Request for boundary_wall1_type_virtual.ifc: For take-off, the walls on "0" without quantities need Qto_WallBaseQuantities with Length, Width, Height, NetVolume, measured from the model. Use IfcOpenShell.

First a look at what the model holds.

```python
import ifcopenshell
import ifcopenshell.util.element
import ifcopenshell.util.unit

model = ifcopenshell.open("boundary_wall1_type_virtual.ifc")
print(model.schema)
for unit_type in ("LENGTHUNIT", "AREAUNIT", "VOLUMEUNIT"):
    print(unit_type, ifcopenshell.util.unit.calculate_unit_scale(model, unit_type))
storey = next(s for s in model.by_type("IfcBuildingStorey") if s.Name == "0")
walls = [e for e in ifcopenshell.util.element.get_decomposition(storey) if e.is_a("IfcWall")]
for e in sorted(walls, key=lambda e: e.id()):
    print(e.id(), e.is_a(), e.Name, list(ifcopenshell.util.element.get_psets(e, qtos_only=True)), sep=" | ")
```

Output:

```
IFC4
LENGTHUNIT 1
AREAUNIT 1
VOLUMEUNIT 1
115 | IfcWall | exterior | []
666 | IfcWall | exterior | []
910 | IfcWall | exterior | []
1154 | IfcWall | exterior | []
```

```python
import ifcopenshell
import ifcopenshell.api.pset
import ifcopenshell.geom
import ifcopenshell.util.element
import ifcopenshell.util.shape
import ifcopenshell.util.unit

model = ifcopenshell.open("boundary_wall1_type_virtual.ifc")
unit_scale = ifcopenshell.util.unit.calculate_unit_scale(model)
volume_scale = ifcopenshell.util.unit.calculate_unit_scale(model, "VOLUMEUNIT")
settings = ifcopenshell.geom.settings()

storey = next(s for s in model.by_type("IfcBuildingStorey") if s.Name == "0")
walls = [e for e in ifcopenshell.util.element.get_decomposition(storey) if e.is_a("IfcWall")]

for e in sorted(walls, key=lambda e: e.id()):
    if ifcopenshell.util.element.get_psets(e, qtos_only=True, should_inherit=False):
        continue
    # Geometry comes back in metres, in the element's own axes.
    shape = ifcopenshell.geom.create_shape(settings, e)
    values = {
        "Length": ifcopenshell.util.shape.get_x(shape.geometry) / unit_scale,
        "Width": ifcopenshell.util.shape.get_y(shape.geometry) / unit_scale,
        "Height": ifcopenshell.util.shape.get_z(shape.geometry) / unit_scale,
        "NetVolume": ifcopenshell.util.shape.get_volume(shape.geometry) / volume_scale,
    }
    qto = ifcopenshell.api.pset.add_qto(model, product=e, name="Qto_WallBaseQuantities")
    ifcopenshell.api.pset.edit_qto(model, qto=qto, properties=values)
    print(e.id(), {k: round(v, 3) for k, v in values.items()})

model.write("boundary_wall1_type_virtual-out.ifc")
```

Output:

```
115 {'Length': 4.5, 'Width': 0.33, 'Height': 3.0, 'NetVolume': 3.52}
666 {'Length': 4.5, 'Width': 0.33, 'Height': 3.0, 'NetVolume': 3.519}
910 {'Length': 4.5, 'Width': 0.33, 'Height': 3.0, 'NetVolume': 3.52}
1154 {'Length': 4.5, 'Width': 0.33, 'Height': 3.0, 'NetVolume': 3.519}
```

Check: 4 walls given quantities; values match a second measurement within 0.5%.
